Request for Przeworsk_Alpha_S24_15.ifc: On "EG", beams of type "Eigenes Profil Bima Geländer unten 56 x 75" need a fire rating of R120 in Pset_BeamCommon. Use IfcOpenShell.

First a look at what the model holds.

```python
import ifcopenshell
import ifcopenshell.util.element

model = ifcopenshell.open("Przeworsk_Alpha_S24_15.ifc")
print(model.schema)
storey = next(s for s in model.by_type("IfcBuildingStorey") if s.Name == "EG")
beams = [e for e in ifcopenshell.util.element.get_decomposition(storey) if e.is_a("IfcBeam")]
seen = {}
for e in beams:
    element_type = ifcopenshell.util.element.get_type(e)
    key = (element_type.Name if element_type != e and element_type else None, ifcopenshell.util.element.get_pset(e, "Pset_BeamCommon", "FireRating"))
    seen[key] = seen.get(key, 0) + 1
for (name, value), count in sorted(seen.items(), key=str):
    print(count, "x", name, "|", value)
```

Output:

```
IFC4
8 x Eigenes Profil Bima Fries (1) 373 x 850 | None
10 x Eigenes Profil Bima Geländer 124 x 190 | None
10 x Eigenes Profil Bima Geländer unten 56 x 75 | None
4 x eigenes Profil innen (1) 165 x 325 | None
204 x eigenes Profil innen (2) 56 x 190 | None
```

```python
import ifcopenshell
import ifcopenshell.api.pset
import ifcopenshell.util.element

model = ifcopenshell.open("Przeworsk_Alpha_S24_15.ifc")

storey = next(s for s in model.by_type("IfcBuildingStorey") if s.Name == "EG")
beams = [e for e in ifcopenshell.util.element.get_decomposition(storey) if e.is_a("IfcBeam")]

count = 0
for e in beams:
    element_type = ifcopenshell.util.element.get_type(e)
    if element_type in (None, e) or element_type.Name != "Eigenes Profil Bima Geländer unten 56 x 75":
        continue
    # add_pset returns the element's existing set when there is one.
    pset = ifcopenshell.api.pset.add_pset(model, product=e, name="Pset_BeamCommon")
    ifcopenshell.api.pset.edit_pset(model, pset=pset, properties={"FireRating": "R120"})
    count += 1

print(count, "beams updated")

model.write("Przeworsk_Alpha_S24_15_v2.ifc")
```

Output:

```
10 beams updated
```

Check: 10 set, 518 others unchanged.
